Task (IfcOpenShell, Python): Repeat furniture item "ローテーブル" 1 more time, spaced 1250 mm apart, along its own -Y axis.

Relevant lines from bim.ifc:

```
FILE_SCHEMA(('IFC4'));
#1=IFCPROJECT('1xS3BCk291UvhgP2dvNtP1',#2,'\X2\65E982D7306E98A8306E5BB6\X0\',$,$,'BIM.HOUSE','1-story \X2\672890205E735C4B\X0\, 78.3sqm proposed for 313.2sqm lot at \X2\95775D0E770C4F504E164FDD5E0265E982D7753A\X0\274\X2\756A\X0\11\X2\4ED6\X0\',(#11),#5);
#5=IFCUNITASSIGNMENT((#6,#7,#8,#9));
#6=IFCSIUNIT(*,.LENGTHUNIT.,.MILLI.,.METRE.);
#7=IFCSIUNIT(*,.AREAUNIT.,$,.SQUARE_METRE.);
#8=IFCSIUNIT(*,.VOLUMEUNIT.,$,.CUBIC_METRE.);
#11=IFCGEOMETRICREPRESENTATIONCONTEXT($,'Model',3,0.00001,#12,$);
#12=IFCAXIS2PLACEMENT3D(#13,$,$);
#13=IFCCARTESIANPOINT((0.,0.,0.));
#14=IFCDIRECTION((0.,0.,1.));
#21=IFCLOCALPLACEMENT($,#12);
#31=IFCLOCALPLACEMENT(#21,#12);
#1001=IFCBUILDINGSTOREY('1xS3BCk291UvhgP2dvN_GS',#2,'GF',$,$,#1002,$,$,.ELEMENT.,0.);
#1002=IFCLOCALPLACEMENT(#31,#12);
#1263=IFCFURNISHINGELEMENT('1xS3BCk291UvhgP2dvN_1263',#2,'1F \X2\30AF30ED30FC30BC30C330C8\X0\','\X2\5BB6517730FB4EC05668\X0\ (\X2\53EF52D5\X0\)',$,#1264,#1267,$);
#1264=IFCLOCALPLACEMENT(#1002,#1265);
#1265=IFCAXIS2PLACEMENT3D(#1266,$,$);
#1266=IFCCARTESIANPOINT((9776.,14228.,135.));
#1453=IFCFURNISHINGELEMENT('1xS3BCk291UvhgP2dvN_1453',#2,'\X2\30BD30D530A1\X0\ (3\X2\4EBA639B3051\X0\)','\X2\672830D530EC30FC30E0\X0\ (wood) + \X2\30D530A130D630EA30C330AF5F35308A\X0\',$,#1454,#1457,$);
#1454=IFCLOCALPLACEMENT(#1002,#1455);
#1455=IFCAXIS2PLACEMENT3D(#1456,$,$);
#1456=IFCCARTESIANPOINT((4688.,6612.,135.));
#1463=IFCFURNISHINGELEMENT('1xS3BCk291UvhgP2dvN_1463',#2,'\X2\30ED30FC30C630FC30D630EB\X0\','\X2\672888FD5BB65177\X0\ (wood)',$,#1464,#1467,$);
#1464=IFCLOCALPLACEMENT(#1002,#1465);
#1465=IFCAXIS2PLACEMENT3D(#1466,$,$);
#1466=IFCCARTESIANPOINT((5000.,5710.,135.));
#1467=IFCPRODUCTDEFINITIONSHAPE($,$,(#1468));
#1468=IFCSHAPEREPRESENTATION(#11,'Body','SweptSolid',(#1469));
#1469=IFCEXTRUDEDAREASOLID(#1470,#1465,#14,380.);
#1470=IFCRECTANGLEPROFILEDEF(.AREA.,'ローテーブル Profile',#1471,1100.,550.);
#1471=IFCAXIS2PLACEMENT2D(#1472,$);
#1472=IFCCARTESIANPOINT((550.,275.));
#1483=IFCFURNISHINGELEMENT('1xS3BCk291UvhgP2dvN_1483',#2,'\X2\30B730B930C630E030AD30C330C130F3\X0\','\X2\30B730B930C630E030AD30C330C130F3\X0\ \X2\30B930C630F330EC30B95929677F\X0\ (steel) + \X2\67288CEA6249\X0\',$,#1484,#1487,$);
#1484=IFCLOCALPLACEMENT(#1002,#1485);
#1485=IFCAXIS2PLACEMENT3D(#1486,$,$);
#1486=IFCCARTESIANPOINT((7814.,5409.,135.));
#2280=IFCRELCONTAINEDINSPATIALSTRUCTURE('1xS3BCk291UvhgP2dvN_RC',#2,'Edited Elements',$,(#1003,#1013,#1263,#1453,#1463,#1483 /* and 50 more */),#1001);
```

```python
import ifcopenshell
import ifcopenshell.api.geometry
import ifcopenshell.api.root
import ifcopenshell.util.element
import ifcopenshell.util.placement

model = ifcopenshell.open("bim.ifc")


def reuse_history(source, copy):
    """copy_class also copies each property set's owner history, people and application; keep the originals."""
    for rel in copy.IsDefinedBy:
        if rel.is_a("IfcRelDefinesByProperties") and (history := rel.RelatingPropertyDefinition.OwnerHistory):
            rel.RelatingPropertyDefinition.OwnerHistory = source.OwnerHistory
            ifcopenshell.util.element.remove_deep2(model, history)


source = model.by_guid("1xS3BCk291UvhgP2dvN_1463")
base = ifcopenshell.util.placement.get_local_placement(source.ObjectPlacement)
step = -base[:3, 1] * 1250.0

for i in range(1, 2):
    copy = ifcopenshell.api.root.copy_class(model, product=source)
    copy.Representation = ifcopenshell.util.element.copy_deep(
        model, source.Representation, exclude=["IfcGeometricRepresentationContext", "IfcRepresentationMap"]
    )
    reuse_history(source, copy)
    matrix = base.copy()
    matrix[:3, 3] += i * step
    print("added at", matrix[:3, 3].round(3) + 0.0)
    ifcopenshell.api.geometry.edit_object_placement(model, product=copy, matrix=matrix, is_si=False)

model.write("bim_edited.ifc")
```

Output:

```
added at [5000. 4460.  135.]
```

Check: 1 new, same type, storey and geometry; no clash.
